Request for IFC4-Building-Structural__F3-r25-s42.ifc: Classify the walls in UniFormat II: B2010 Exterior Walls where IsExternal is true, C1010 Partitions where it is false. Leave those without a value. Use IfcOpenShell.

First a look at what the model holds.

```python
import ifcopenshell
import ifcopenshell.util.element

model = ifcopenshell.open("IFC4-Building-Structural__F3-r25-s42.ifc")
print(model.schema)
print("classifications:", [c.Name for c in model.by_type("IfcClassification")])
values = [ifcopenshell.util.element.get_pset(e, "Pset_WallCommon", "IsExternal") for e in model.by_type("IfcWall")]
for value in (True, False, None):
    print("IsExternal", value, values.count(value))
```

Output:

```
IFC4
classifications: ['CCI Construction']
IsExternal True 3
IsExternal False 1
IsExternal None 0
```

```python
import ifcopenshell
import ifcopenshell.api.classification
import ifcopenshell.util.element

model = ifcopenshell.open("IFC4-Building-Structural__F3-r25-s42.ifc")

system = ifcopenshell.api.classification.add_classification(model, classification="UniFormat II")

walls = model.by_type("IfcWall")
external = {e: ifcopenshell.util.element.get_pset(e, "Pset_WallCommon", "IsExternal") for e in walls}
for flag, code, name in ((True, "B2010", "Exterior Walls"), (False, "C1010", "Partitions")):
    products = [e for e in walls if external[e] is flag]
    ifcopenshell.api.classification.add_reference(
        model, products=products, classification=system, identification=code, name=name
    )
    print(code, len(products))

model.write("IFC4-Building-Structural__F3-r25-s42_v2.ifc")
```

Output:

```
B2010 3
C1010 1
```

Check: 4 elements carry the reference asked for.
